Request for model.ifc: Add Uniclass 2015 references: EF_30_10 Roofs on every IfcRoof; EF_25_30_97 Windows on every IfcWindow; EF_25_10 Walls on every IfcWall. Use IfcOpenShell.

First a look at what the model holds.

```python
import ifcopenshell

model = ifcopenshell.open("model.ifc")
print(model.schema)
print("classifications:", [c.Name for c in model.by_type("IfcClassification")])
for ifc_class in ("IfcDoor", "IfcRoof", "IfcStair", "IfcWall", "IfcWindow"):
    print(ifc_class, len(model.by_type(ifc_class)))
```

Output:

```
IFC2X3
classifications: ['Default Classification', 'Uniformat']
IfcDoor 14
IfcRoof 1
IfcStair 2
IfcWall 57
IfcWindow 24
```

```python
import ifcopenshell
import ifcopenshell.api.classification

model = ifcopenshell.open("model.ifc")

# IFC2X3 requires Source and Edition and has no link from the project to the system.
system = model.create_entity("IfcClassification", Source="NBS", Edition="2015", Name="Uniclass 2015")

codes = {
    "IfcRoof": ("EF_30_10", "Roofs"),
    "IfcWindow": ("EF_25_30_97", "Windows"),
    "IfcWall": ("EF_25_10", "Walls"),
}
for ifc_class, (code, name) in codes.items():
    products = model.by_type(ifc_class)
    ifcopenshell.api.classification.add_reference(
        model, products=products, classification=system, identification=code, name=name
    )
    print(code, len(products))

model.write("model_rev.ifc")
```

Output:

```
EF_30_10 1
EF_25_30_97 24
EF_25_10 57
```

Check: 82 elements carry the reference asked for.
